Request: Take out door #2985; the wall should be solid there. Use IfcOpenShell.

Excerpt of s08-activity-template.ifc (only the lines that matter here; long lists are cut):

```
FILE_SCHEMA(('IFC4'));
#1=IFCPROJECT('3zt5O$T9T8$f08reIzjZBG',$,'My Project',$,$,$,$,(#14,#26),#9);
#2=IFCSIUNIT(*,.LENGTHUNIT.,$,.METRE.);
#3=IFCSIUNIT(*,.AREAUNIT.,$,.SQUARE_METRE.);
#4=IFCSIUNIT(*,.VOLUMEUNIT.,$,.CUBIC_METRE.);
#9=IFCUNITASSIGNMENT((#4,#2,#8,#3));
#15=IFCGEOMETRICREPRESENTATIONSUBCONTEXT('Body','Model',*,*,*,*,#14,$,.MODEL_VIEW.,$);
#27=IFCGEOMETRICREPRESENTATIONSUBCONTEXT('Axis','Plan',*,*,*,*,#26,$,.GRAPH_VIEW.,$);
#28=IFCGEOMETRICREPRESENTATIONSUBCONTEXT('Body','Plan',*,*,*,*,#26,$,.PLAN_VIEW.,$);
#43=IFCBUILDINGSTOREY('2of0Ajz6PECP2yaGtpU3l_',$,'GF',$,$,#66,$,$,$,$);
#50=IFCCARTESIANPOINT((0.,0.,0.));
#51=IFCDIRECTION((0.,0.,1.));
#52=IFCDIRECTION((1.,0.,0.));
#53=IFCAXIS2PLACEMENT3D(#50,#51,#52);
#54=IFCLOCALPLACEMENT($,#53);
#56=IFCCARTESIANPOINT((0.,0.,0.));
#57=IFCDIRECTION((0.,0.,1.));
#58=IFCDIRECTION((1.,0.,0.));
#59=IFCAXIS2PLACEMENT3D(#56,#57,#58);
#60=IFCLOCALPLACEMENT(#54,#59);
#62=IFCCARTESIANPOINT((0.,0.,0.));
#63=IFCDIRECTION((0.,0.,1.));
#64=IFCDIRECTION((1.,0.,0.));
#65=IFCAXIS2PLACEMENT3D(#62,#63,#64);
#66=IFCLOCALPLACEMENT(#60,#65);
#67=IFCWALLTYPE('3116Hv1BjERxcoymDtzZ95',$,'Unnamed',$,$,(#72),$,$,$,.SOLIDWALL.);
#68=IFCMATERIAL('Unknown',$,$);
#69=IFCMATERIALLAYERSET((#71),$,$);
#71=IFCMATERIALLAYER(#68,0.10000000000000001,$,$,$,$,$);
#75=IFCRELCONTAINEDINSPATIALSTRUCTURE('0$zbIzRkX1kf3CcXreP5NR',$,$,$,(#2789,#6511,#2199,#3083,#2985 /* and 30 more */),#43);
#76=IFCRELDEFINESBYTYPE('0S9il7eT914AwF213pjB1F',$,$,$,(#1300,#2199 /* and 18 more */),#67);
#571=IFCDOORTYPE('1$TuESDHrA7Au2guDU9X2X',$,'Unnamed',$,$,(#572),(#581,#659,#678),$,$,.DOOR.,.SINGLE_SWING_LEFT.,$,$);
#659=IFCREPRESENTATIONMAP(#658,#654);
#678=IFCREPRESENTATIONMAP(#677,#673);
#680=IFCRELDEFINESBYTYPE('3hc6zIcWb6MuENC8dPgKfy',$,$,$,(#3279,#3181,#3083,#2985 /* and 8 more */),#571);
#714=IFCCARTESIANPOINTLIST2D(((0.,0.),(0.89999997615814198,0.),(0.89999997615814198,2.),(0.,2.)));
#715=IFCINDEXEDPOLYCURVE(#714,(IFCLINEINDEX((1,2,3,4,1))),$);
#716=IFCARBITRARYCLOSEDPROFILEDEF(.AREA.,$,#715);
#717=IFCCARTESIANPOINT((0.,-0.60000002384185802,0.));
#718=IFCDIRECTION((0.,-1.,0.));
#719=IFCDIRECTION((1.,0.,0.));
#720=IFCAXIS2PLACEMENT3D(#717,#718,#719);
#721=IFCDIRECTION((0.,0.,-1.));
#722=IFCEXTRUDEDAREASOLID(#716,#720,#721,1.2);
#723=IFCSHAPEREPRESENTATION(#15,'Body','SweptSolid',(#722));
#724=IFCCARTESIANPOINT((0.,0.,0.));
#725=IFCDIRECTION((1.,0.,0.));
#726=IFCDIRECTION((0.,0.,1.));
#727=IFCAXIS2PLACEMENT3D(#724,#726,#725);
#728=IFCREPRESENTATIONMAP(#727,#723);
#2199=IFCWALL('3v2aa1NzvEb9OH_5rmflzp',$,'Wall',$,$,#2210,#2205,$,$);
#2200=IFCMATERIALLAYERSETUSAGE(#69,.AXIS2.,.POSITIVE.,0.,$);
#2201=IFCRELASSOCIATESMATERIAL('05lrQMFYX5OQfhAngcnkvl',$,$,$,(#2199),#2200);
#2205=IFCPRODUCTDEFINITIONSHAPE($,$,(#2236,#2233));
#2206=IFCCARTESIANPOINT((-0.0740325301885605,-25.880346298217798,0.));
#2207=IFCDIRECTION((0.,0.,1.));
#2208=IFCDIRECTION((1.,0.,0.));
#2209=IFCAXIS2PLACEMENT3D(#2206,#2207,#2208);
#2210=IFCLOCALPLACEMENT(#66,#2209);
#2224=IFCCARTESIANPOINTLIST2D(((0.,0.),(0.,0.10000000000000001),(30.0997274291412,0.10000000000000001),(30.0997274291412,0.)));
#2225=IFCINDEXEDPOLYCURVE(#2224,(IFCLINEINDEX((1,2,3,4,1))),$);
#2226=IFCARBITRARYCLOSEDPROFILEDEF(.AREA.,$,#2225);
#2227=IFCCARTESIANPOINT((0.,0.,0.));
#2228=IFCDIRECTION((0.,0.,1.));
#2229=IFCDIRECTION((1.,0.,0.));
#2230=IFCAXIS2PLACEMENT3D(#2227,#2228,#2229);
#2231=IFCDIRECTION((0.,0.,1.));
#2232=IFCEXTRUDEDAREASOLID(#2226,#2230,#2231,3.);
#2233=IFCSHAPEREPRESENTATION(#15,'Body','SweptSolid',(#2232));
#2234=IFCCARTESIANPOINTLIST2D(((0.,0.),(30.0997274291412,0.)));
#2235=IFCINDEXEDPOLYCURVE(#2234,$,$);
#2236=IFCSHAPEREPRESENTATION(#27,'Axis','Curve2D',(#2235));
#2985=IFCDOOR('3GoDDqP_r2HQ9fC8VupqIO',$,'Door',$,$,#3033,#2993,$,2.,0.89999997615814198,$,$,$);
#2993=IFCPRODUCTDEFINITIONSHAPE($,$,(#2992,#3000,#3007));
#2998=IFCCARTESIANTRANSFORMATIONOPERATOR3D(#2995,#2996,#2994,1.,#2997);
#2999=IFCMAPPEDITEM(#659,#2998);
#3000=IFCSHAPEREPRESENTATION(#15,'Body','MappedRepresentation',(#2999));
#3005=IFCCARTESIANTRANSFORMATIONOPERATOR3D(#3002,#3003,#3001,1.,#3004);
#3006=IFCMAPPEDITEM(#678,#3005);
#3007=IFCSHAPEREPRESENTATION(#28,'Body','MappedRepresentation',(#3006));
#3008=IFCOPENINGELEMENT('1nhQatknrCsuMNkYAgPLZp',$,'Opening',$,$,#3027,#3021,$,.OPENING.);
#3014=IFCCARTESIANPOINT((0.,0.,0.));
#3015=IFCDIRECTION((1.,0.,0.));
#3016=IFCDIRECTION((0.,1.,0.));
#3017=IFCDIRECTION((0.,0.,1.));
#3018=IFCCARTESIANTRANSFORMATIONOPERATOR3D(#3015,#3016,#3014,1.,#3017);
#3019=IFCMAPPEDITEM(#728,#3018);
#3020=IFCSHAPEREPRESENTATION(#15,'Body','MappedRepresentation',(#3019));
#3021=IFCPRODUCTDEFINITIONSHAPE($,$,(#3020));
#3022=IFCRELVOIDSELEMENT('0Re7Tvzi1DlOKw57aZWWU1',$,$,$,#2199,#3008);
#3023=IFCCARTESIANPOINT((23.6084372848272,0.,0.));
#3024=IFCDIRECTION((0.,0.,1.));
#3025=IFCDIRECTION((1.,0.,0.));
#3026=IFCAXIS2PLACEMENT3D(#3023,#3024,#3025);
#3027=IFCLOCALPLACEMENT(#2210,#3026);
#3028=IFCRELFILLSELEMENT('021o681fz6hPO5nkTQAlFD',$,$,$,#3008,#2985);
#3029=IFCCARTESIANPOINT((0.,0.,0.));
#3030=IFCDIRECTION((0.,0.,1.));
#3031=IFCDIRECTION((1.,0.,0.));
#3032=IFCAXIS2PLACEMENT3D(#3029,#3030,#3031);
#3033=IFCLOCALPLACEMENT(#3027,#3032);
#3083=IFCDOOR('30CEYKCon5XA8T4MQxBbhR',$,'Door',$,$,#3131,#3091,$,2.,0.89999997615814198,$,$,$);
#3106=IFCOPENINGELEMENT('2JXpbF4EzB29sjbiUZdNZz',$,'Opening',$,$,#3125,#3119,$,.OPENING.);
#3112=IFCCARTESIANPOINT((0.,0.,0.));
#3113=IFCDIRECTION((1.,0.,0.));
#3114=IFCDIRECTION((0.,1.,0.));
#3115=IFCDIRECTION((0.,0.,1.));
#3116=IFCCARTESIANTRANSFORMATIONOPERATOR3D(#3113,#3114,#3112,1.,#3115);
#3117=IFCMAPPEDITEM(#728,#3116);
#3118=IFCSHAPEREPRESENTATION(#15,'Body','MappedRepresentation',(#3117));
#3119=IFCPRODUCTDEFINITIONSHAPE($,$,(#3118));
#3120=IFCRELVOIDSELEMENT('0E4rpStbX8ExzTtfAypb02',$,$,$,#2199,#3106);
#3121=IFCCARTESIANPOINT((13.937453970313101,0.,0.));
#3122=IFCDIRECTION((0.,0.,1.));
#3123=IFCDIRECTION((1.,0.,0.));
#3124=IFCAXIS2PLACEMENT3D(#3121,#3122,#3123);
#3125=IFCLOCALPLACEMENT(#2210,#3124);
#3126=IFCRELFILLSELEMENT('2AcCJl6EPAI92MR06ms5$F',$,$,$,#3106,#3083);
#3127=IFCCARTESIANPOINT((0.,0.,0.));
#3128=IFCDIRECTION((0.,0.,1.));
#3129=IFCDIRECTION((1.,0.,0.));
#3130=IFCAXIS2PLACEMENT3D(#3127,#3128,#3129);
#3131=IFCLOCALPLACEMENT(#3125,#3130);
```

```python
import ifcopenshell
import ifcopenshell.api.feature
import ifcopenshell.api.root
import ifcopenshell.geom
import ifcopenshell.util.shape

model = ifcopenshell.open("s08-activity-template.ifc")
settings = ifcopenshell.geom.settings()


def volume(element):
    """Net volume in cubic metres, openings subtracted."""
    shape = ifcopenshell.geom.create_shape(settings, element)
    return ifcopenshell.util.shape.get_volume(shape.geometry)


door = model.by_guid("3GoDDqP_r2HQ9fC8VupqIO")
opening = door.FillsVoids[0].RelatingOpeningElement
wall = opening.VoidsElements[0].RelatingBuildingElement
before = volume(wall)

ifcopenshell.api.root.remove_product(model, product=door)
ifcopenshell.api.feature.remove_feature(model, feature=opening)

after = volume(wall)

print(f"wall volume {before:.3f} -> {after:.3f} m3")

model.write("s08-activity-template_v2.ifc")
```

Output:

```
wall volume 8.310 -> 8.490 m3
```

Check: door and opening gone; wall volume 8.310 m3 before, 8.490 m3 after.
